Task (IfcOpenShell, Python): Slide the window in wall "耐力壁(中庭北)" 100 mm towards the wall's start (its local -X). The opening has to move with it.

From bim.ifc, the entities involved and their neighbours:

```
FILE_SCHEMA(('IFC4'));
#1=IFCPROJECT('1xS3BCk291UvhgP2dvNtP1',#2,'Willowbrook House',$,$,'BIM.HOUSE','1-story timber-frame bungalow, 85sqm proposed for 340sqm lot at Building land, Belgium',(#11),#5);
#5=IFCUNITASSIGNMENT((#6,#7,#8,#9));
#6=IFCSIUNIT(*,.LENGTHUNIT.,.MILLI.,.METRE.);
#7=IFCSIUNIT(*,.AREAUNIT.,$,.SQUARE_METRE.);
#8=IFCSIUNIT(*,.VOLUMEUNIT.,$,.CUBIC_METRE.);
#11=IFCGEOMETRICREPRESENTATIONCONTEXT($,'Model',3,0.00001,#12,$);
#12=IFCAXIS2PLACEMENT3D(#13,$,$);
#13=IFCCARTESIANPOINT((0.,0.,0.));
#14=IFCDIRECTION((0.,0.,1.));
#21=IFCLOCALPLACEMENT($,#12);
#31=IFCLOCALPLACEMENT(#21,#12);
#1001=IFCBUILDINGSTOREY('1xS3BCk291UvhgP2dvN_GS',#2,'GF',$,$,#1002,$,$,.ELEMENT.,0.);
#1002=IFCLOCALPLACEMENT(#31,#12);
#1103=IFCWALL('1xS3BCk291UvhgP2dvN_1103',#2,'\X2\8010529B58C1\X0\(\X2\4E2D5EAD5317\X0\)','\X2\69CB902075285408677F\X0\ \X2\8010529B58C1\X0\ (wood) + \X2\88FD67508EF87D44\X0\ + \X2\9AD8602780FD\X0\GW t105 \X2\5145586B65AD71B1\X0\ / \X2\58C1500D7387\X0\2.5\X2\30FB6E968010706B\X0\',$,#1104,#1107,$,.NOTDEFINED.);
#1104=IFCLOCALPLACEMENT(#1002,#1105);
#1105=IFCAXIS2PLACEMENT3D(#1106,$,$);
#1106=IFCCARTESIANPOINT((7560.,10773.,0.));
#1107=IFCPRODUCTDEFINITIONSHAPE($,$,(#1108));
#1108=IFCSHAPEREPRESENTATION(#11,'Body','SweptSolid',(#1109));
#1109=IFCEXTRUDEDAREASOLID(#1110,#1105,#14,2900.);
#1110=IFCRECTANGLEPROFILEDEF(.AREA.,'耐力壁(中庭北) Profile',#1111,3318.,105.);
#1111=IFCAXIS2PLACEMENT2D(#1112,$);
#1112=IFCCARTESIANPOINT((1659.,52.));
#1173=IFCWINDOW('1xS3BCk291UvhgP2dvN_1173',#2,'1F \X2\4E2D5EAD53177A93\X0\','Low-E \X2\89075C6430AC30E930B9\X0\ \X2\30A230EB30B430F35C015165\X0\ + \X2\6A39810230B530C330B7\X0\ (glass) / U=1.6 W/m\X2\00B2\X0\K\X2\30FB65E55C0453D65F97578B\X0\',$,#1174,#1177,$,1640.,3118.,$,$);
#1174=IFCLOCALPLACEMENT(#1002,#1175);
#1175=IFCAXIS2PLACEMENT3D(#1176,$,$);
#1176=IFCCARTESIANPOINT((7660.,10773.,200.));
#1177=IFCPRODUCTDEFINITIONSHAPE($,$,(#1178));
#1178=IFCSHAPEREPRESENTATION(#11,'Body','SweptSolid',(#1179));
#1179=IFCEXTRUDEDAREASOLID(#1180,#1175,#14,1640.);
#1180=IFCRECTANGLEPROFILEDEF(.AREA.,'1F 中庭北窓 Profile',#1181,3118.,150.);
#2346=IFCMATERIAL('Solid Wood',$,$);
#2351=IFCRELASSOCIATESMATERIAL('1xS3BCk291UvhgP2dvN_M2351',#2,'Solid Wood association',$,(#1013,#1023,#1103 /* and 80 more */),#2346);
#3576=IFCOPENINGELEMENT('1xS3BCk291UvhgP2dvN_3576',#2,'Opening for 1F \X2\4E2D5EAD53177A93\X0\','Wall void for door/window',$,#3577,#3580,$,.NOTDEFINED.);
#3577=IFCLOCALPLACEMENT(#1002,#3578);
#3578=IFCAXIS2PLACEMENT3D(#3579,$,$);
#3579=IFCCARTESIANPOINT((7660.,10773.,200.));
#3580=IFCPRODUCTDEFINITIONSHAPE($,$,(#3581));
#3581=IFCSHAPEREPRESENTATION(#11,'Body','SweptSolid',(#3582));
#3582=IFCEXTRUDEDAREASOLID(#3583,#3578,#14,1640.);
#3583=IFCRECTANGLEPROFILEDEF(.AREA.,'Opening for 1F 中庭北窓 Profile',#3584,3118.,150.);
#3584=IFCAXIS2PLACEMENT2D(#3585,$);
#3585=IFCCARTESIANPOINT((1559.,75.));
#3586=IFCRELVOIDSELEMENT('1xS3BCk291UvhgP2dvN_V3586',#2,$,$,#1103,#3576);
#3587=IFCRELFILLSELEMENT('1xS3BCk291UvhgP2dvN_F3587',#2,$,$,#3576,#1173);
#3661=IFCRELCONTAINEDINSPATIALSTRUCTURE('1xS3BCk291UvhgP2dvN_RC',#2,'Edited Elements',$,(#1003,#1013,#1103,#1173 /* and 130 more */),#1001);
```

```python
import ifcopenshell
import ifcopenshell.api.geometry
import ifcopenshell.util.placement
import ifcopenshell.util.unit

model = ifcopenshell.open("bim.ifc")
unit_scale = ifcopenshell.util.unit.calculate_unit_scale(model)

window = model.by_guid("1xS3BCk291UvhgP2dvN_1173")
opening = window.FillsVoids[0].RelatingOpeningElement
wall = opening.VoidsElements[0].RelatingBuildingElement

wall_matrix = ifcopenshell.util.placement.get_local_placement(wall.ObjectPlacement)
shift = wall_matrix[:3, 0] * -0.1 / unit_scale
before = ifcopenshell.util.placement.get_local_placement(window.ObjectPlacement)[:3, 3].copy()

# The window is not placed relative to its opening, so move both.
for product in (opening, window):
    matrix = ifcopenshell.util.placement.get_local_placement(product.ObjectPlacement)
    matrix[:3, 3] += shift
    ifcopenshell.api.geometry.edit_object_placement(model, product=product, matrix=matrix, is_si=False)

after = ifcopenshell.util.placement.get_local_placement(window.ObjectPlacement)[:3, 3]
print("window moved by", (after - before).round(3) + 0.0)

model.write("bim-out.ifc")
```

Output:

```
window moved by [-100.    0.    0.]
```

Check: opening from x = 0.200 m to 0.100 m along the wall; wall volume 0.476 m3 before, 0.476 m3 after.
